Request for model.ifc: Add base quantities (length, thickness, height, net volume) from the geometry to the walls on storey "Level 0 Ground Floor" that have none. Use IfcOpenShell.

First a look at what the model holds.

```python
import ifcopenshell
import ifcopenshell.util.element
import ifcopenshell.util.unit

model = ifcopenshell.open("model.ifc")
print(model.schema)
for unit_type in ("LENGTHUNIT", "AREAUNIT", "VOLUMEUNIT"):
    print(unit_type, ifcopenshell.util.unit.calculate_unit_scale(model, unit_type))
storey = next(s for s in model.by_type("IfcBuildingStorey") if s.Name == "Level 0 Ground Floor")
walls = [e for e in ifcopenshell.util.element.get_decomposition(storey) if e.is_a("IfcWall")]
for e in sorted(walls, key=lambda e: e.id()):
    print(e.id(), e.is_a(), e.Name, list(ifcopenshell.util.element.get_psets(e, qtos_only=True)), sep=" | ")
```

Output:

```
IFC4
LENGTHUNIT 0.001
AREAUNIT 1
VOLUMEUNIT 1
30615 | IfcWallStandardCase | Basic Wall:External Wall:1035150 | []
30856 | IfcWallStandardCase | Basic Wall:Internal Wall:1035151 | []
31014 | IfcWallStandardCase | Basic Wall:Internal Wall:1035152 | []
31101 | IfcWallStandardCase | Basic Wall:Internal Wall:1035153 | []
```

```python
import ifcopenshell
import ifcopenshell.api.pset
import ifcopenshell.geom
import ifcopenshell.util.element
import ifcopenshell.util.shape
import ifcopenshell.util.unit

model = ifcopenshell.open("model.ifc")
unit_scale = ifcopenshell.util.unit.calculate_unit_scale(model)
volume_scale = ifcopenshell.util.unit.calculate_unit_scale(model, "VOLUMEUNIT")
settings = ifcopenshell.geom.settings()

storey = next(s for s in model.by_type("IfcBuildingStorey") if s.Name == "Level 0 Ground Floor")
walls = [e for e in ifcopenshell.util.element.get_decomposition(storey) if e.is_a("IfcWall")]

for e in sorted(walls, key=lambda e: e.id()):
    if ifcopenshell.util.element.get_psets(e, qtos_only=True, should_inherit=False):
        continue
    # Geometry comes back in metres, in the element's own axes.
    shape = ifcopenshell.geom.create_shape(settings, e)
    values = {
        "Length": ifcopenshell.util.shape.get_x(shape.geometry) / unit_scale,
        "Width": ifcopenshell.util.shape.get_y(shape.geometry) / unit_scale,
        "Height": ifcopenshell.util.shape.get_z(shape.geometry) / unit_scale,
        "NetVolume": ifcopenshell.util.shape.get_volume(shape.geometry) / volume_scale,
    }
    qto = ifcopenshell.api.pset.add_qto(model, product=e, name="Qto_WallBaseQuantities")
    ifcopenshell.api.pset.edit_qto(model, qto=qto, properties=values)
    print(e.id(), {k: round(v, 3) for k, v in values.items()})

model.write("model_edited.ifc")
```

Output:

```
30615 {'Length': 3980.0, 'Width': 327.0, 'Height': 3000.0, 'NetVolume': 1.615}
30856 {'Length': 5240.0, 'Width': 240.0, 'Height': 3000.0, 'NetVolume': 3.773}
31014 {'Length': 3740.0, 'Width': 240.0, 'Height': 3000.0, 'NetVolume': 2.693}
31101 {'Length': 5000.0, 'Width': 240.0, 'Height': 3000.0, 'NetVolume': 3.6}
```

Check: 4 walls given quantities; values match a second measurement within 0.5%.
